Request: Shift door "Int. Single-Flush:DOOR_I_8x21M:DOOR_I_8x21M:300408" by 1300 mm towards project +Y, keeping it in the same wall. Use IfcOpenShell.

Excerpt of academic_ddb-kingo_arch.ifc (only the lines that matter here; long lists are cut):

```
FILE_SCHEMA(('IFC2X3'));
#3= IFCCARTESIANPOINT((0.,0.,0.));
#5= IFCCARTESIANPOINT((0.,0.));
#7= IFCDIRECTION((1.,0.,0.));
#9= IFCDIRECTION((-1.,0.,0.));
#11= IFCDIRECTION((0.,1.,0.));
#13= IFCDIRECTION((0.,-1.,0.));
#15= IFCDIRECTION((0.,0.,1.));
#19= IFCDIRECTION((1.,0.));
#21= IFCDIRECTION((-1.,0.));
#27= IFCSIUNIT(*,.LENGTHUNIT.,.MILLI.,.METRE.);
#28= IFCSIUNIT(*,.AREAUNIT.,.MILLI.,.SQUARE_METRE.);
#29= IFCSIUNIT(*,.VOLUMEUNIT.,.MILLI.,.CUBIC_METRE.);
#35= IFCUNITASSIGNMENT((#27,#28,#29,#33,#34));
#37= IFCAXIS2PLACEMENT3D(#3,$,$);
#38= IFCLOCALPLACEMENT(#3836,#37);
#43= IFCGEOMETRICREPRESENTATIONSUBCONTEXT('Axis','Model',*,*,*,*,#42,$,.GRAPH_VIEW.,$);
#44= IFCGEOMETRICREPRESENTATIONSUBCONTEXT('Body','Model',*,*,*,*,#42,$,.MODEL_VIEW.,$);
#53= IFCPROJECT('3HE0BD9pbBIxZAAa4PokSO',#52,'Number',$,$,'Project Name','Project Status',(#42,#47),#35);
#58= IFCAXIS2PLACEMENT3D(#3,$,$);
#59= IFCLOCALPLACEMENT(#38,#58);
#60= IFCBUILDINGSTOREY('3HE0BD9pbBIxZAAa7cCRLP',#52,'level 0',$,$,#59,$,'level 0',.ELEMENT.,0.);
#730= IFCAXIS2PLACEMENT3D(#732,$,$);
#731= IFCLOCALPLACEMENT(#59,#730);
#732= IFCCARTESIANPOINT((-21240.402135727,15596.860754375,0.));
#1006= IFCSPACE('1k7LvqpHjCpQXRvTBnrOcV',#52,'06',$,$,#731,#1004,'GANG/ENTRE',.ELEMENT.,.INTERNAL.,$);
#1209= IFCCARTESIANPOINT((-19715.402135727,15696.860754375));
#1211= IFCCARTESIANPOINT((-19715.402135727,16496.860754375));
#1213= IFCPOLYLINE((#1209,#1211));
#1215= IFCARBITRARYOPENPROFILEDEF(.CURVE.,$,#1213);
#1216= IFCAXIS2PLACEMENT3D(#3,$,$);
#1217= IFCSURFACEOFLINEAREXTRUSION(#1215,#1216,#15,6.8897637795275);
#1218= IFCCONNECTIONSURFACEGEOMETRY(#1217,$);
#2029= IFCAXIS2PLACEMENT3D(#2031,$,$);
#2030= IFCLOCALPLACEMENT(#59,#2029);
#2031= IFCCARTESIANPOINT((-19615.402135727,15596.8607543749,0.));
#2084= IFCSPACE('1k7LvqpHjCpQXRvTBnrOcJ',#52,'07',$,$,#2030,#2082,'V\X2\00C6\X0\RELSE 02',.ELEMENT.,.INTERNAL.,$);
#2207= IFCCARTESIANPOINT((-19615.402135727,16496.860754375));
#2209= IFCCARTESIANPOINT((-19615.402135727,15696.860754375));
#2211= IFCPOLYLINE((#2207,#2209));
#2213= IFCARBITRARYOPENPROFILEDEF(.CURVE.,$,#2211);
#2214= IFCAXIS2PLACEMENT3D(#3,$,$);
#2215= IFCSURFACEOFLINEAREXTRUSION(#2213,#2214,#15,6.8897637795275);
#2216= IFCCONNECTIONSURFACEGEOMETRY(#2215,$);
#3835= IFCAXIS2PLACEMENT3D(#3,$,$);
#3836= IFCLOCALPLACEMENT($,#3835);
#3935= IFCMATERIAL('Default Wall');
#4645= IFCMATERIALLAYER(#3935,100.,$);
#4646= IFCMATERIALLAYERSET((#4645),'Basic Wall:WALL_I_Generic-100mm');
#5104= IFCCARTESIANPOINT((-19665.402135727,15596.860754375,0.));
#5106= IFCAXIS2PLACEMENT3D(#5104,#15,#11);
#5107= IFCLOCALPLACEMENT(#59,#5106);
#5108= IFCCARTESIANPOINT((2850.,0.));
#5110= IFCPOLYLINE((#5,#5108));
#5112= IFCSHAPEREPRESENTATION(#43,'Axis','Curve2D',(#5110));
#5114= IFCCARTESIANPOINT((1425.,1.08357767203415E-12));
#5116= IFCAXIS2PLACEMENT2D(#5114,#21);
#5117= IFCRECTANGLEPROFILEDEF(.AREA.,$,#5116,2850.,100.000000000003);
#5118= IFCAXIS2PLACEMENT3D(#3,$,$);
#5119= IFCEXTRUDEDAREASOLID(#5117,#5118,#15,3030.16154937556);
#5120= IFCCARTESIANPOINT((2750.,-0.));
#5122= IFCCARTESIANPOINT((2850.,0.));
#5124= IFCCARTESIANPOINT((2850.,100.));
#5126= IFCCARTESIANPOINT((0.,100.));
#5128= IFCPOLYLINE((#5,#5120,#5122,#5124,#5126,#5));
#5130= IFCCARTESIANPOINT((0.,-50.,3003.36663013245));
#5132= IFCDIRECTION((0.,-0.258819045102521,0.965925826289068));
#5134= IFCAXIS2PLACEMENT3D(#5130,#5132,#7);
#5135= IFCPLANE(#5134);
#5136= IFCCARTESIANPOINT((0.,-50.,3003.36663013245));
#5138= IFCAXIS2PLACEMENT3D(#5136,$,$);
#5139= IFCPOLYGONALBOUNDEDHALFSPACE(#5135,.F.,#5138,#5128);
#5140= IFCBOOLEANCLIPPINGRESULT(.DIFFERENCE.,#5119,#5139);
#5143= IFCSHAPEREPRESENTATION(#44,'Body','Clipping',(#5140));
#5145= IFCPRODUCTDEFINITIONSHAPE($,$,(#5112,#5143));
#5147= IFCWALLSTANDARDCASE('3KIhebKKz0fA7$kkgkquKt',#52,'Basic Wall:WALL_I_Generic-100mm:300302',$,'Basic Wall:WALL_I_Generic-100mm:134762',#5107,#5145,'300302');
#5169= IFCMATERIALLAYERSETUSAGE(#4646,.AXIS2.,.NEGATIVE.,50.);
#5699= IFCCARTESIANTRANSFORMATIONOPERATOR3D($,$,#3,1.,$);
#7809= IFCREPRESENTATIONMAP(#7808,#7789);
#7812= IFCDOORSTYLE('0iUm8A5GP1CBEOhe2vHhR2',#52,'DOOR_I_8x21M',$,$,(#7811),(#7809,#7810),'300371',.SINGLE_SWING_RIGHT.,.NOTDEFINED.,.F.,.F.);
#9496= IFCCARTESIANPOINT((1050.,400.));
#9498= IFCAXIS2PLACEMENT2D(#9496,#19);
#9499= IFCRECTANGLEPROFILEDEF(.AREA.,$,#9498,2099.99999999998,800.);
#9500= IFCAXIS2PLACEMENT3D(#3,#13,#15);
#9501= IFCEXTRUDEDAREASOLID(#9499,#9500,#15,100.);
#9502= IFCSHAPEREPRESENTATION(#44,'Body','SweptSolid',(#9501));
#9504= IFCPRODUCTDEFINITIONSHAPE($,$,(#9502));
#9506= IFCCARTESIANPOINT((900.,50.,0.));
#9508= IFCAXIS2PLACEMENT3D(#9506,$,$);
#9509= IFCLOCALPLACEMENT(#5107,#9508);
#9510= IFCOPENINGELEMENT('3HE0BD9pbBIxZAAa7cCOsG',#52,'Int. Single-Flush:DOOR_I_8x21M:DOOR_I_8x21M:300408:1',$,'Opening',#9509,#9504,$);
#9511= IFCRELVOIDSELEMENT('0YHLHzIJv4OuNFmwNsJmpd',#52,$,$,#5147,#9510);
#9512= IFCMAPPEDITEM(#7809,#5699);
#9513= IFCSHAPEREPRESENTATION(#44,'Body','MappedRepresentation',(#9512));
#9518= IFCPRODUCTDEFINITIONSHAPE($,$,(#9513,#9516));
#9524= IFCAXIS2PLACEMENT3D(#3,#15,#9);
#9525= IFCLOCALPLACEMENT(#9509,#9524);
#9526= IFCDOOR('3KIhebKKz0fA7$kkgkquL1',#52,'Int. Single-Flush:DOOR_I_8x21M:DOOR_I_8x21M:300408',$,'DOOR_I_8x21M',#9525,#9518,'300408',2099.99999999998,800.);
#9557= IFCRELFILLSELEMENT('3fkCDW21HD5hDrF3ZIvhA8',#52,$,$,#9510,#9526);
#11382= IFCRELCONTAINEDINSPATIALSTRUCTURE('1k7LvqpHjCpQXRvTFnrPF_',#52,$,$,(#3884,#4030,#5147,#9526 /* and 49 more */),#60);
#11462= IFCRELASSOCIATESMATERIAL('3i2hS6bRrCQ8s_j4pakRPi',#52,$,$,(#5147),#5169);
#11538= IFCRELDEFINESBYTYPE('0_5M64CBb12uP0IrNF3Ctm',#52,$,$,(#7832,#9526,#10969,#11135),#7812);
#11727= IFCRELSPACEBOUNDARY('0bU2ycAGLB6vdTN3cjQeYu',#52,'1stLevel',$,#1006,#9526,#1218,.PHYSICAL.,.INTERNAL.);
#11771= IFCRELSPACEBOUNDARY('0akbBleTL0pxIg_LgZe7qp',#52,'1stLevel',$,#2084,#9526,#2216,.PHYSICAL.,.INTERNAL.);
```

```python
import numpy as np
import ifcopenshell
import ifcopenshell.api.geometry
import ifcopenshell.util.placement
import ifcopenshell.util.unit

model = ifcopenshell.open("academic_ddb-kingo_arch.ifc")
unit_scale = ifcopenshell.util.unit.calculate_unit_scale(model)

door = model.by_guid("3KIhebKKz0fA7$kkgkquL1")
opening = door.FillsVoids[0].RelatingOpeningElement
wall = opening.VoidsElements[0].RelatingBuildingElement

wall_matrix = ifcopenshell.util.placement.get_local_placement(wall.ObjectPlacement)
shift = wall_matrix[:3, 0] * 1.3 / unit_scale
before = ifcopenshell.util.placement.get_local_placement(door.ObjectPlacement)[:3, 3].copy()

# The door is placed relative to its opening, so it follows when the opening moves.
matrix = ifcopenshell.util.placement.get_local_placement(opening.ObjectPlacement)
matrix[:3, 3] += shift
ifcopenshell.api.geometry.edit_object_placement(
    model, product=opening, matrix=matrix, is_si=False, should_transform_children=True
)

# Space boundary surfaces are stored in each space's coordinates; move them too.
for rel in door.ProvidesBoundaries:
    if not rel.ConnectionGeometry:
        continue
    surface = rel.ConnectionGeometry.SurfaceOnRelatingElement
    space_matrix = ifcopenshell.util.placement.get_local_placement(rel.RelatingSpace.ObjectPlacement)
    point = np.array(surface.Position.Location.Coordinates) + space_matrix[:3, :3].T @ shift
    surface.Position = model.createIfcAxis2Placement3D(
        model.createIfcCartesianPoint(point.tolist()), surface.Position.Axis, surface.Position.RefDirection
    )

after = ifcopenshell.util.placement.get_local_placement(door.ObjectPlacement)[:3, 3]
print("door moved by", (after - before).round(3) + 0.0)

model.write("academic_ddb-kingo_arch_edited.ifc")
```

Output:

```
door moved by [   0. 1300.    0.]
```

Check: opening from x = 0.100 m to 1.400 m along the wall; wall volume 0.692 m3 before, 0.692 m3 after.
